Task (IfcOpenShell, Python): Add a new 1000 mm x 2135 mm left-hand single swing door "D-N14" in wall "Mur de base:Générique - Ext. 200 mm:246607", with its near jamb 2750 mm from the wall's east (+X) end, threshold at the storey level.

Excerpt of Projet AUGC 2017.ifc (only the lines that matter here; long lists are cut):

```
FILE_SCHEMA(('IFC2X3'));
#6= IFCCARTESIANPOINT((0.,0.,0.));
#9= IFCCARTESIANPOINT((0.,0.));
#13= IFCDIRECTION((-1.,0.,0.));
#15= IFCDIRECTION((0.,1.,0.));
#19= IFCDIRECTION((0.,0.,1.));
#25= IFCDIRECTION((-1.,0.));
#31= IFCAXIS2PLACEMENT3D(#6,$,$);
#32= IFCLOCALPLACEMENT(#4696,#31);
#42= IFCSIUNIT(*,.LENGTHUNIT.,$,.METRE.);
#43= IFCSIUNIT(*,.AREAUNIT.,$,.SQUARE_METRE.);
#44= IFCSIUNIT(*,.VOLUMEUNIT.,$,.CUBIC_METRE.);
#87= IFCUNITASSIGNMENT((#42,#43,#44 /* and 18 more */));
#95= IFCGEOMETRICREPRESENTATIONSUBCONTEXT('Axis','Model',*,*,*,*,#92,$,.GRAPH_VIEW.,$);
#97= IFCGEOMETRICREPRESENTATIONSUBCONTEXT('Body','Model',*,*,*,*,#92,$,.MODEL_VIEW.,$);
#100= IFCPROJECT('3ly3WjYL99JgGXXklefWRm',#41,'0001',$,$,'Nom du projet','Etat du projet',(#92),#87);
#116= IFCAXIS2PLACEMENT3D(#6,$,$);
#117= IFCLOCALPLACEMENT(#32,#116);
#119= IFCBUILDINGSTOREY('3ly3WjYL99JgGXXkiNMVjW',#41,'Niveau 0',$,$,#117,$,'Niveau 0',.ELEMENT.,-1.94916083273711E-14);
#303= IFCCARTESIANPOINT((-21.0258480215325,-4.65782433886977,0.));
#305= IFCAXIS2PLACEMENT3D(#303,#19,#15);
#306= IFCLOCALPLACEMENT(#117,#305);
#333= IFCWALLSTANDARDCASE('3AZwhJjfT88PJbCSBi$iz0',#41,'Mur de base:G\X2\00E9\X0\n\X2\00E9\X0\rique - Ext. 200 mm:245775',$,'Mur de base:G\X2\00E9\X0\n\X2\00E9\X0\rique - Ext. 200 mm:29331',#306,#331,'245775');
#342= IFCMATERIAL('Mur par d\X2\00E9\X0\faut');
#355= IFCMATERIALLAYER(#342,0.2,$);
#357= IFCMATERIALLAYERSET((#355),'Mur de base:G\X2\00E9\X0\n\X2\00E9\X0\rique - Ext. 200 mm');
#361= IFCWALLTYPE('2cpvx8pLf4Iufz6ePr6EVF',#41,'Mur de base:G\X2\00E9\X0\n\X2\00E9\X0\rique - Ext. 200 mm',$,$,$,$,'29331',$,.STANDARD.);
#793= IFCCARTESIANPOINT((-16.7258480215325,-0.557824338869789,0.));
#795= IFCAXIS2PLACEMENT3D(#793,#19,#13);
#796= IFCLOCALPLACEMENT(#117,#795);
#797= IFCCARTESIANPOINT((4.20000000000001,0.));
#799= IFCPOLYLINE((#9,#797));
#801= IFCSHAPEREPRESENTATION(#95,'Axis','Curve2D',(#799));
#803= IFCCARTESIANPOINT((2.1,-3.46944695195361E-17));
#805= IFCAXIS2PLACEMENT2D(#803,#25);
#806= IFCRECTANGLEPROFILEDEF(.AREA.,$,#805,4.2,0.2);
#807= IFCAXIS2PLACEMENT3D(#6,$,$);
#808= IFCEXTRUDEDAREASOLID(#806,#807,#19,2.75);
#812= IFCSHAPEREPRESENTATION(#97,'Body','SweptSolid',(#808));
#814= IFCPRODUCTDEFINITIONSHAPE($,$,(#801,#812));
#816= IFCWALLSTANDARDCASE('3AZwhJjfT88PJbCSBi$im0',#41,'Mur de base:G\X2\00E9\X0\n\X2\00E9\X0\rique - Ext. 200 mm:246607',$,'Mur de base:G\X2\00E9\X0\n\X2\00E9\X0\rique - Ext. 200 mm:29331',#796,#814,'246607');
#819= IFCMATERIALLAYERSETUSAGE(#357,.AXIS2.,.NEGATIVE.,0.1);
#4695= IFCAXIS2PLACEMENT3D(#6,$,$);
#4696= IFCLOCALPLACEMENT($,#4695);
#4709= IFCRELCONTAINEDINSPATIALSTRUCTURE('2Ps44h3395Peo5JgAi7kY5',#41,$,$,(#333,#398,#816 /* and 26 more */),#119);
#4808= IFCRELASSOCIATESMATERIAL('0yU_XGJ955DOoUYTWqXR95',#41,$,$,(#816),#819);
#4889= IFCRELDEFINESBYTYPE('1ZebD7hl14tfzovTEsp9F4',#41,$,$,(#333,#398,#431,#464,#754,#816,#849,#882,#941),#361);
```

```python
import numpy as np
import ifcopenshell
import ifcopenshell.api.feature
import ifcopenshell.api.geometry
import ifcopenshell.api.root
import ifcopenshell.api.spatial
import ifcopenshell.api.type
import ifcopenshell.geom
import ifcopenshell.util.element
import ifcopenshell.util.placement
import ifcopenshell.util.representation
import ifcopenshell.util.shape
import ifcopenshell.util.unit

model = ifcopenshell.open("Projet AUGC 2017.ifc")
unit_scale = ifcopenshell.util.unit.calculate_unit_scale(model)
settings = ifcopenshell.geom.settings()


def volume(element):
    """Net volume in cubic metres, openings subtracted."""
    shape = ifcopenshell.geom.create_shape(settings, element)
    return ifcopenshell.util.shape.get_volume(shape.geometry)


wall = model.by_guid("3AZwhJjfT88PJbCSBi$im0")
storey = ifcopenshell.util.element.get_container(wall, ifc_class="IfcBuildingStorey")
context = ifcopenshell.util.representation.get_context(model, "Model", "Body", "MODEL_VIEW")
before = volume(wall)

width, height, from_end, sill = 1, 2.135, 2.75, 0.0  # metres

# The wall runs along its own X axis, and the end named is its -X end.
wall_shape = ifcopenshell.geom.create_shape(settings, wall)
x, y, z = ifcopenshell.util.shape.get_vertices(wall_shape.geometry).T
start = x.min() + from_end
face, thickness = float(y.min()), float(y.max() - y.min())
wall_matrix = ifcopenshell.util.placement.get_local_placement(wall.ObjectPlacement)
level = ifcopenshell.util.placement.get_local_placement(storey.ObjectPlacement)[2, 3]


def in_wall(x, y):
    """Placement at x, y metres in the wall's axes, at sill height."""
    matrix = wall_matrix.copy()
    matrix[:, 3] = wall_matrix @ np.array([x / unit_scale, y / unit_scale, 0.0, 1.0])
    matrix[2, 3] = level + sill / unit_scale
    return matrix


# Opening: a box that overshoots both wall faces by 50 mm.
opening = ifcopenshell.api.root.create_entity(model, ifc_class="IfcOpeningElement")
box = ifcopenshell.api.geometry.add_wall_representation(
    model, context=context, length=width, height=height, thickness=thickness + 0.1
)
ifcopenshell.api.geometry.assign_representation(model, product=opening, representation=box)
ifcopenshell.api.geometry.edit_object_placement(model, product=opening, matrix=in_wall(start, face - 0.05), is_si=False)
ifcopenshell.api.feature.add_feature(model, feature=opening, element=wall)

door = ifcopenshell.api.root.create_entity(model, ifc_class="IfcDoor", name="D-N14")
door.OverallWidth, door.OverallHeight = width / unit_scale, height / unit_scale
body = ifcopenshell.api.geometry.add_door_representation(
    model,
    context=context,
    overall_width=door.OverallWidth,
    overall_height=door.OverallHeight,
    operation_type="SINGLE_SWING_LEFT",
    lining_properties={"LiningDepth": thickness / unit_scale, "ThresholdDepth": thickness / unit_scale},
)
ifcopenshell.api.geometry.assign_representation(model, product=door, representation=body)
ifcopenshell.api.spatial.assign_container(model, products=[door], relating_structure=storey)
fills = ifcopenshell.api.feature.add_filling(model, opening=opening, element=door)
fills.OwnerHistory = door.OwnerHistory  # required in IFC2X3

# IFC2X3 keeps the operation on the door style.
style = ifcopenshell.api.root.create_entity(model, ifc_class="IfcDoorStyle", name="D-N14")
style.OperationType, style.ConstructionType = "SINGLE_SWING_LEFT", "NOTDEFINED"
style.ParameterTakesPrecedence = style.Sizeable = False
ifcopenshell.api.type.assign_type(model, related_objects=[door], relating_type=style)

# The lining spans the wall, so the door starts at the wall face.
ifcopenshell.api.geometry.edit_object_placement(model, product=door, matrix=in_wall(start, face), is_si=False)

after = volume(wall)

print(f"wall volume {before:.3f} -> {after:.3f} m3")

model.write("Projet AUGC 2017_v2.ifc")
```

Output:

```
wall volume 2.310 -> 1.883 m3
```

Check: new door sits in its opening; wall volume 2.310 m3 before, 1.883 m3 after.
